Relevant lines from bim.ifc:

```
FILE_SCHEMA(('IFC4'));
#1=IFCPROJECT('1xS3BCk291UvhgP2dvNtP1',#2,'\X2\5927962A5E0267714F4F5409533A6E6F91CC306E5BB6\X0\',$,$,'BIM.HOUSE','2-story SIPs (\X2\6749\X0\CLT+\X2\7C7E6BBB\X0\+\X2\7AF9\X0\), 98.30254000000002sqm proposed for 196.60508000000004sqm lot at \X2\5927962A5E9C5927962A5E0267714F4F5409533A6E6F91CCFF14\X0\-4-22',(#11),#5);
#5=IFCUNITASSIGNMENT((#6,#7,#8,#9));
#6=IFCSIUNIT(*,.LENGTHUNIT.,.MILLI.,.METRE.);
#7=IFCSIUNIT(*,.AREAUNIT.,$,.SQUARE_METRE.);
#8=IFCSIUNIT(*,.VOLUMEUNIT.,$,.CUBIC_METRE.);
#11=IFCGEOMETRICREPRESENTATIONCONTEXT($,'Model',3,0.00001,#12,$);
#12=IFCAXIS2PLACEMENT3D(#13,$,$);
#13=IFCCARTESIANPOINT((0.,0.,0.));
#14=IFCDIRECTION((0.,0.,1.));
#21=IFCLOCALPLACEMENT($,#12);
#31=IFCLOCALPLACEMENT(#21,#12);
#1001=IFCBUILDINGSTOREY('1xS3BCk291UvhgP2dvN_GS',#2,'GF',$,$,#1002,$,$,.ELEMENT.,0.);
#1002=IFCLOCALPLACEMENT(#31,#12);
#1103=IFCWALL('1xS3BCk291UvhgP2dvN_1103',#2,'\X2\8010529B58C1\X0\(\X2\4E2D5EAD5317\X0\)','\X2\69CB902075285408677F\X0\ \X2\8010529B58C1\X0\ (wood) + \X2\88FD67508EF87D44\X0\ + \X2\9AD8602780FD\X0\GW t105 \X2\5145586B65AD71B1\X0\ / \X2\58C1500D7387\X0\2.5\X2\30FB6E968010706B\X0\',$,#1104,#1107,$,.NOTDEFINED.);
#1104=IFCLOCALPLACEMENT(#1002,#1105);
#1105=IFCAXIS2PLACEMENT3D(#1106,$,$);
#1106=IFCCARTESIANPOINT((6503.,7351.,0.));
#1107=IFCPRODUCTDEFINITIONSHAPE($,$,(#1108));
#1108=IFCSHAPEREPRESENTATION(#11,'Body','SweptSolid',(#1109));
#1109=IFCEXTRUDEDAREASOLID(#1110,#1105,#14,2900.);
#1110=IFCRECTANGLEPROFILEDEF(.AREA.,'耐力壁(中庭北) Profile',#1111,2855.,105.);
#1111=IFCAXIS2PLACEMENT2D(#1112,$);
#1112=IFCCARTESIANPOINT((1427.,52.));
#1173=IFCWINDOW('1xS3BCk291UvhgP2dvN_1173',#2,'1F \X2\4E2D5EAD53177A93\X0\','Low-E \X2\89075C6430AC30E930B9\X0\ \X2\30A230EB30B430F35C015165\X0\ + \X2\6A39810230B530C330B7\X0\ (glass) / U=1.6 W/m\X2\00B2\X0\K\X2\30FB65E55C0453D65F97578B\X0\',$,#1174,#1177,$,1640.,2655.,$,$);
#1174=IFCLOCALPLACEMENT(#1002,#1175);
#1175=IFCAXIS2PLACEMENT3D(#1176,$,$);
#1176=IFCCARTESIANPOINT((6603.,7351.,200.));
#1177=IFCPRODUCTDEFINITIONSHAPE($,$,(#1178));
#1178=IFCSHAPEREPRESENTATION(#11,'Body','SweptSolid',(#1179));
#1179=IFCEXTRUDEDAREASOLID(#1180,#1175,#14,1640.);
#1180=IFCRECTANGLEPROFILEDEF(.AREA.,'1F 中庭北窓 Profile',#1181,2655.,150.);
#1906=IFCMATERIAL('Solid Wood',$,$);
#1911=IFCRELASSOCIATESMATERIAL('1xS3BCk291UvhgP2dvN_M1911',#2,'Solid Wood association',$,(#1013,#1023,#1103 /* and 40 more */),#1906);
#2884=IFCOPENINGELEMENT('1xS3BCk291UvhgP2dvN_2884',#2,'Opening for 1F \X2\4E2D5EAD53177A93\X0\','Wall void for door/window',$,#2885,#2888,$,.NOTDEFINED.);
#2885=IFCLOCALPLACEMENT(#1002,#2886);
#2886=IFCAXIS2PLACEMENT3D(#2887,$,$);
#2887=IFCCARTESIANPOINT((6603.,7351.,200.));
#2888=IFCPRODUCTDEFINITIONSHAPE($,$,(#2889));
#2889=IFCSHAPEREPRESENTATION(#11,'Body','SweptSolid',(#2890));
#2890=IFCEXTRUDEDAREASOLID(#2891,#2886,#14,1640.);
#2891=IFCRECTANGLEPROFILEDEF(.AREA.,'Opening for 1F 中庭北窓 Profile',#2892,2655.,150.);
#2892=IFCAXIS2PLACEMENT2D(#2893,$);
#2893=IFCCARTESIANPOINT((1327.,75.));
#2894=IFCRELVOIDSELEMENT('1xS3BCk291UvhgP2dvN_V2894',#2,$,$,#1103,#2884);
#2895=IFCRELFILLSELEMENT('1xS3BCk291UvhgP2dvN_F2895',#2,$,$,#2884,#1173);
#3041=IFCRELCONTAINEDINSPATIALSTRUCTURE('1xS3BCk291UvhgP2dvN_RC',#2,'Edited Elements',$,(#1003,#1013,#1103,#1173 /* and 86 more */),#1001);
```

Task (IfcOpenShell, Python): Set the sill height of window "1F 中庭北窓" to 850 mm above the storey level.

```python
import numpy as np
import ifcopenshell
import ifcopenshell.api.geometry
import ifcopenshell.geom
import ifcopenshell.util.element
import ifcopenshell.util.placement
import ifcopenshell.util.shape
import ifcopenshell.util.unit

model = ifcopenshell.open("bim.ifc")
unit_scale = ifcopenshell.util.unit.calculate_unit_scale(model)

window = model.by_guid("1xS3BCk291UvhgP2dvN_1173")
opening = window.FillsVoids[0].RelatingOpeningElement
storey = ifcopenshell.util.element.get_container(window, ifc_class="IfcBuildingStorey")
level = ifcopenshell.util.placement.get_local_placement(storey.ObjectPlacement)[2, 3]

# The opening's origin need not be at the sill, so measure its lowest point.
shape = ifcopenshell.geom.create_shape(ifcopenshell.geom.settings(), opening)
bottom = ifcopenshell.util.shape.get_shape_bottom_elevation(shape, shape.geometry) / unit_scale
dz = level + 850.0 - bottom

shift = np.array([0.0, 0.0, dz])
# The window is not placed relative to its opening, so move both.
for product in (opening, window):
    matrix = ifcopenshell.util.placement.get_local_placement(product.ObjectPlacement)
    matrix[:3, 3] += shift
    ifcopenshell.api.geometry.edit_object_placement(model, product=product, matrix=matrix, is_si=False)

print(f"moved by {dz * unit_scale:+.3f} m")

model.write("bim_updated.ifc")
```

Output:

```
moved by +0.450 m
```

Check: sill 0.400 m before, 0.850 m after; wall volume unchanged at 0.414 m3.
